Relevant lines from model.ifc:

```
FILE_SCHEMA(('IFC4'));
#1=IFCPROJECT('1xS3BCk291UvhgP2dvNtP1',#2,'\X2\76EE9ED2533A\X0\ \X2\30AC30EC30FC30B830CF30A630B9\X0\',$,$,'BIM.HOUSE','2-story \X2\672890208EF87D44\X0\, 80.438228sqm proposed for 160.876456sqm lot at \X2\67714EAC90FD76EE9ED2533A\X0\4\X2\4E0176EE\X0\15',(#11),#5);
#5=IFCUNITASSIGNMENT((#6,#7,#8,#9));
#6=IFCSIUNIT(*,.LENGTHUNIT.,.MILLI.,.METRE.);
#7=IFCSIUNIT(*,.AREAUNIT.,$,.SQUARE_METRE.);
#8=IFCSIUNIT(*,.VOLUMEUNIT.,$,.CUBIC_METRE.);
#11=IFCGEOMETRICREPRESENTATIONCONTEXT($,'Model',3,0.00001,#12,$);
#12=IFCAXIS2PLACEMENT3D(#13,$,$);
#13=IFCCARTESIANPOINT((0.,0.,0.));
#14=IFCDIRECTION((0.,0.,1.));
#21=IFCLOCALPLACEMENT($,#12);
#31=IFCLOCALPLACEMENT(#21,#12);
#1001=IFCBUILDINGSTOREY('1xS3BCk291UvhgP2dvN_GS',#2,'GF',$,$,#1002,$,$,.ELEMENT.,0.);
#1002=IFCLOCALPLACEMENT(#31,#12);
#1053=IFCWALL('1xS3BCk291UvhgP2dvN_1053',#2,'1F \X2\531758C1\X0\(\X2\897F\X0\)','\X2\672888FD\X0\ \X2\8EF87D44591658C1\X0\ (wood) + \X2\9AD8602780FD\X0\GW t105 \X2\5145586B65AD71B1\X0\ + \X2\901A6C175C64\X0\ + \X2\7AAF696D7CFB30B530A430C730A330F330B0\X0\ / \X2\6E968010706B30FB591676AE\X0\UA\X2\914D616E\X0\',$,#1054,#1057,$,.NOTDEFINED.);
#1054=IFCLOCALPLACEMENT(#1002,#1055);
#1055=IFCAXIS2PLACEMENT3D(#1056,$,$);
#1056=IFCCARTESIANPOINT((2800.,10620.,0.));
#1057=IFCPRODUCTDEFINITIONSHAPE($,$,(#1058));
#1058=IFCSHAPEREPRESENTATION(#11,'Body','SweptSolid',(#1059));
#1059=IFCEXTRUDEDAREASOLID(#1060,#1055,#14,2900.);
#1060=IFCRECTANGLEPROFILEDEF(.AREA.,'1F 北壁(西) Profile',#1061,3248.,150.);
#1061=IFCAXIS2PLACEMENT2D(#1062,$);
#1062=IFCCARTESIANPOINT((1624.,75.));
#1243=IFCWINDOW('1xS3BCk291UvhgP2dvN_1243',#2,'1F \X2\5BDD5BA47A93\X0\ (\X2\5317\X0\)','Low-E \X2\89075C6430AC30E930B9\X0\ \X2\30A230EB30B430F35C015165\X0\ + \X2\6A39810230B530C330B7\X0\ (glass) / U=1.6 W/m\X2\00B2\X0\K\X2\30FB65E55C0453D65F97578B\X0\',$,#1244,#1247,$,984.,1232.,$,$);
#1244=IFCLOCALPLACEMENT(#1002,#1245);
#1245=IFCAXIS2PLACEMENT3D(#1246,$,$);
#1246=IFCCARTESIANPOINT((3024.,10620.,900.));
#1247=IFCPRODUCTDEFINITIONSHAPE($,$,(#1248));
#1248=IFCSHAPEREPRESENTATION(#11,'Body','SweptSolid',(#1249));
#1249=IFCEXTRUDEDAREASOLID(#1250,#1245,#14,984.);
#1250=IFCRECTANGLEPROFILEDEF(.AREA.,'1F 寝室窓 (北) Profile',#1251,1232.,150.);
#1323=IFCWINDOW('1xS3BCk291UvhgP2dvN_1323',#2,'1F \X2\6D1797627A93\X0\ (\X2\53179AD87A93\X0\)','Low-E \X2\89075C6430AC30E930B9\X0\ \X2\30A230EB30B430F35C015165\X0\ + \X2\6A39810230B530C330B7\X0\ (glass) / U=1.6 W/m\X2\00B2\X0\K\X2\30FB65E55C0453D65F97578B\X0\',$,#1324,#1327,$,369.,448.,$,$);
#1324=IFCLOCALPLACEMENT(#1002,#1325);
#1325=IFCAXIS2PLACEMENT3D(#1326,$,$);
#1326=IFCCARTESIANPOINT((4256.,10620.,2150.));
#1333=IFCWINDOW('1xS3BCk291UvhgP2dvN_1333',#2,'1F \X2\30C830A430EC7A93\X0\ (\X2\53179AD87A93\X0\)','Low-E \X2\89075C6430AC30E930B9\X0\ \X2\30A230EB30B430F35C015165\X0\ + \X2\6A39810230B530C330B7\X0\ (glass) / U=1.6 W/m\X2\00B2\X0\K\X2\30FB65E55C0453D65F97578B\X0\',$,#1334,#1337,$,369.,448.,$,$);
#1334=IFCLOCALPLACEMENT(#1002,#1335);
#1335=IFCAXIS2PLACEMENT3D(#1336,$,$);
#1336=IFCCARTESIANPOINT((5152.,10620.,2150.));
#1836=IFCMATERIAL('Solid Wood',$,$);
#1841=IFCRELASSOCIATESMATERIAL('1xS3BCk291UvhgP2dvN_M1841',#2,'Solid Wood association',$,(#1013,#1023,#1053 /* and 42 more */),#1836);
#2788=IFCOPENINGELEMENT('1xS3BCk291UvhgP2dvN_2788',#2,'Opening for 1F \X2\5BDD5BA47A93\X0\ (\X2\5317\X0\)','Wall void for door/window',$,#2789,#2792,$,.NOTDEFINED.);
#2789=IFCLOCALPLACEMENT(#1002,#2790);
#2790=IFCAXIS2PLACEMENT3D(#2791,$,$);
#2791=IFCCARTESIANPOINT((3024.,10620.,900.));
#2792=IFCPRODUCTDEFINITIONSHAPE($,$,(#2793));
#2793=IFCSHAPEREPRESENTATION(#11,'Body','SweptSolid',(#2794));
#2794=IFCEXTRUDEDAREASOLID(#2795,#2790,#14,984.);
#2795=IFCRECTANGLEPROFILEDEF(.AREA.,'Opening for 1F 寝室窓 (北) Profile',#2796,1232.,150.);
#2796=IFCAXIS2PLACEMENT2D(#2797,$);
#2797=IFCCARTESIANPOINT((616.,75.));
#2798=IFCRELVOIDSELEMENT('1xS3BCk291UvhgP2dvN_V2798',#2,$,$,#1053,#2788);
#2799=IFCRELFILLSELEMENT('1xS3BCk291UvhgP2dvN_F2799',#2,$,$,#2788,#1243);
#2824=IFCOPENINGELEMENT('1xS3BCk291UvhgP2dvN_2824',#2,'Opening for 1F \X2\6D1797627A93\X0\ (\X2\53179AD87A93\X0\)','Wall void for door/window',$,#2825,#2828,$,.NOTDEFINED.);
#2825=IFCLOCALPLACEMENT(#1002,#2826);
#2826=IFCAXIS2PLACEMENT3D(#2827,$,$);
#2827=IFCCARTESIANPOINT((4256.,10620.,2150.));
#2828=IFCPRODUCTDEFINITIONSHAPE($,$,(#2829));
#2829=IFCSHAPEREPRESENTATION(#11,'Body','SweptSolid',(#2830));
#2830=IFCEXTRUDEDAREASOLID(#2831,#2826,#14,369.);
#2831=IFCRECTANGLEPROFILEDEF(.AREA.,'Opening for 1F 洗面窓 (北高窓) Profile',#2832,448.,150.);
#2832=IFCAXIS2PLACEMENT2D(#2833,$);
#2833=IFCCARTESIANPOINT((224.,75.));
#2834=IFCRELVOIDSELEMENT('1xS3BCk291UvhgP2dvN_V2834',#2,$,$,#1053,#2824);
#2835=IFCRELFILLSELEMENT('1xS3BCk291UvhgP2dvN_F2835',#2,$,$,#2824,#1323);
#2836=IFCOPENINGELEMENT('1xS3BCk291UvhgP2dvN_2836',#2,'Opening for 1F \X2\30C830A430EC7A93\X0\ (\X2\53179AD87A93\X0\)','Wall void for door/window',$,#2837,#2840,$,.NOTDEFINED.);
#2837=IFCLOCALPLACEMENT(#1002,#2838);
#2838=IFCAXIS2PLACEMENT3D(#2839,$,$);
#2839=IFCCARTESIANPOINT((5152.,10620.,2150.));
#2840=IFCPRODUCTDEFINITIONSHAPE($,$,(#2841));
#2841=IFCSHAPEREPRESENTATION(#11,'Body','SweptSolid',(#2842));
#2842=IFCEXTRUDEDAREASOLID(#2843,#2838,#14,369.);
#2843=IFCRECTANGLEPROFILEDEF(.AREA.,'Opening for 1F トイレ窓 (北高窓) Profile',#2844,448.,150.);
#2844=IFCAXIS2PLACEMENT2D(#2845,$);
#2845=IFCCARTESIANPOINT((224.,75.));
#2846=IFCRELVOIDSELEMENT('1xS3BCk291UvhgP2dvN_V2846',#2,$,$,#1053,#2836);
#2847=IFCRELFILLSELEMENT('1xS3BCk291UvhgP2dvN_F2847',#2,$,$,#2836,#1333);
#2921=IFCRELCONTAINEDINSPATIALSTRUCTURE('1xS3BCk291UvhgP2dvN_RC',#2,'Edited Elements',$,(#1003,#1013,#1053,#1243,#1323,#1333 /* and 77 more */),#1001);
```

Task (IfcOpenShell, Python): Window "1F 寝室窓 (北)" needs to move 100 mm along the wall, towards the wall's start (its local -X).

```python
import ifcopenshell
import ifcopenshell.api.geometry
import ifcopenshell.util.placement
import ifcopenshell.util.unit

model = ifcopenshell.open("model.ifc")
unit_scale = ifcopenshell.util.unit.calculate_unit_scale(model)

window = model.by_guid("1xS3BCk291UvhgP2dvN_1243")
opening = window.FillsVoids[0].RelatingOpeningElement
wall = opening.VoidsElements[0].RelatingBuildingElement

wall_matrix = ifcopenshell.util.placement.get_local_placement(wall.ObjectPlacement)
shift = wall_matrix[:3, 0] * -0.1 / unit_scale
before = ifcopenshell.util.placement.get_local_placement(window.ObjectPlacement)[:3, 3].copy()

# The window is not placed relative to its opening, so move both.
for product in (opening, window):
    matrix = ifcopenshell.util.placement.get_local_placement(product.ObjectPlacement)
    matrix[:3, 3] += shift
    ifcopenshell.api.geometry.edit_object_placement(model, product=product, matrix=matrix, is_si=False)

after = ifcopenshell.util.placement.get_local_placement(window.ObjectPlacement)[:3, 3]
print("window moved by", (after - before).round(3) + 0.0)

model.write("model_v2.ifc")
```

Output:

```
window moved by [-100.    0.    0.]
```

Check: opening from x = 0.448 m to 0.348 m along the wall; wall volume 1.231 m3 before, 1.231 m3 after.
